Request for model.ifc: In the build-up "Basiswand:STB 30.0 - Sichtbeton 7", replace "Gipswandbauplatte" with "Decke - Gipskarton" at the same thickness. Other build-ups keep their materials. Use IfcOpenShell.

First a look at what the model holds.

```python
import ifcopenshell
import ifcopenshell.util.element

model = ifcopenshell.open("model.ifc")
print(model.schema)
for layer_set in model.by_type("IfcMaterialLayerSet"):
    if layer_set.LayerSetName == "Basiswand:STB 30.0 - Sichtbeton 7":
        for layer in layer_set.MaterialLayers:
            print(layer.id(), layer.Material and layer.Material.Name, layer.LayerThickness, sep=" | ")
        print(len(ifcopenshell.util.element.get_elements_by_material(model, layer_set)), "elements and types use it")
print(sorted(m.Name for m in model.by_type("IfcMaterial") if m.Name)[:60])
```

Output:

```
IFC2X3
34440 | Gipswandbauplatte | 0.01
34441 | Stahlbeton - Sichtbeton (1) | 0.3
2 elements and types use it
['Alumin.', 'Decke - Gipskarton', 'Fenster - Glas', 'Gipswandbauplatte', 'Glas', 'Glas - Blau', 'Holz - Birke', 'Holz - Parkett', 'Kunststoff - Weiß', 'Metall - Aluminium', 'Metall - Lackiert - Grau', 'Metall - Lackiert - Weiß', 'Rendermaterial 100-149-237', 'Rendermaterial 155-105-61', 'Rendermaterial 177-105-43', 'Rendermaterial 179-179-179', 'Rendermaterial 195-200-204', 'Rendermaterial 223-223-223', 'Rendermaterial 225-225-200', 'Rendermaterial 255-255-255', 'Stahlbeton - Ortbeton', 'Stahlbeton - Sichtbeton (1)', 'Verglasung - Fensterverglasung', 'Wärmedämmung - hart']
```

```python
import ifcopenshell
import ifcopenshell.api.material

model = ifcopenshell.open("model.ifc")

layer_set = next(s for s in model.by_type("IfcMaterialLayerSet") if s.LayerSetName == "Basiswand:STB 30.0 - Sichtbeton 7")
layer = next(l for l in layer_set.MaterialLayers if l.Material and l.Material.Name == "Gipswandbauplatte")
material = next(m for m in model.by_type("IfcMaterial") if m.Name == "Decke - Gipskarton")

# Point this one layer at the other material; renaming the old one would change it everywhere.
ifcopenshell.api.material.edit_layer(model, layer=layer, attributes={}, material=material)

print([l.Material.Name if l.Material else None for l in layer_set.MaterialLayers])

model.write("model_updated.ifc")
```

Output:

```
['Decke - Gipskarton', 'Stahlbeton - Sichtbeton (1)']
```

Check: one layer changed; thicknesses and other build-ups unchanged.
